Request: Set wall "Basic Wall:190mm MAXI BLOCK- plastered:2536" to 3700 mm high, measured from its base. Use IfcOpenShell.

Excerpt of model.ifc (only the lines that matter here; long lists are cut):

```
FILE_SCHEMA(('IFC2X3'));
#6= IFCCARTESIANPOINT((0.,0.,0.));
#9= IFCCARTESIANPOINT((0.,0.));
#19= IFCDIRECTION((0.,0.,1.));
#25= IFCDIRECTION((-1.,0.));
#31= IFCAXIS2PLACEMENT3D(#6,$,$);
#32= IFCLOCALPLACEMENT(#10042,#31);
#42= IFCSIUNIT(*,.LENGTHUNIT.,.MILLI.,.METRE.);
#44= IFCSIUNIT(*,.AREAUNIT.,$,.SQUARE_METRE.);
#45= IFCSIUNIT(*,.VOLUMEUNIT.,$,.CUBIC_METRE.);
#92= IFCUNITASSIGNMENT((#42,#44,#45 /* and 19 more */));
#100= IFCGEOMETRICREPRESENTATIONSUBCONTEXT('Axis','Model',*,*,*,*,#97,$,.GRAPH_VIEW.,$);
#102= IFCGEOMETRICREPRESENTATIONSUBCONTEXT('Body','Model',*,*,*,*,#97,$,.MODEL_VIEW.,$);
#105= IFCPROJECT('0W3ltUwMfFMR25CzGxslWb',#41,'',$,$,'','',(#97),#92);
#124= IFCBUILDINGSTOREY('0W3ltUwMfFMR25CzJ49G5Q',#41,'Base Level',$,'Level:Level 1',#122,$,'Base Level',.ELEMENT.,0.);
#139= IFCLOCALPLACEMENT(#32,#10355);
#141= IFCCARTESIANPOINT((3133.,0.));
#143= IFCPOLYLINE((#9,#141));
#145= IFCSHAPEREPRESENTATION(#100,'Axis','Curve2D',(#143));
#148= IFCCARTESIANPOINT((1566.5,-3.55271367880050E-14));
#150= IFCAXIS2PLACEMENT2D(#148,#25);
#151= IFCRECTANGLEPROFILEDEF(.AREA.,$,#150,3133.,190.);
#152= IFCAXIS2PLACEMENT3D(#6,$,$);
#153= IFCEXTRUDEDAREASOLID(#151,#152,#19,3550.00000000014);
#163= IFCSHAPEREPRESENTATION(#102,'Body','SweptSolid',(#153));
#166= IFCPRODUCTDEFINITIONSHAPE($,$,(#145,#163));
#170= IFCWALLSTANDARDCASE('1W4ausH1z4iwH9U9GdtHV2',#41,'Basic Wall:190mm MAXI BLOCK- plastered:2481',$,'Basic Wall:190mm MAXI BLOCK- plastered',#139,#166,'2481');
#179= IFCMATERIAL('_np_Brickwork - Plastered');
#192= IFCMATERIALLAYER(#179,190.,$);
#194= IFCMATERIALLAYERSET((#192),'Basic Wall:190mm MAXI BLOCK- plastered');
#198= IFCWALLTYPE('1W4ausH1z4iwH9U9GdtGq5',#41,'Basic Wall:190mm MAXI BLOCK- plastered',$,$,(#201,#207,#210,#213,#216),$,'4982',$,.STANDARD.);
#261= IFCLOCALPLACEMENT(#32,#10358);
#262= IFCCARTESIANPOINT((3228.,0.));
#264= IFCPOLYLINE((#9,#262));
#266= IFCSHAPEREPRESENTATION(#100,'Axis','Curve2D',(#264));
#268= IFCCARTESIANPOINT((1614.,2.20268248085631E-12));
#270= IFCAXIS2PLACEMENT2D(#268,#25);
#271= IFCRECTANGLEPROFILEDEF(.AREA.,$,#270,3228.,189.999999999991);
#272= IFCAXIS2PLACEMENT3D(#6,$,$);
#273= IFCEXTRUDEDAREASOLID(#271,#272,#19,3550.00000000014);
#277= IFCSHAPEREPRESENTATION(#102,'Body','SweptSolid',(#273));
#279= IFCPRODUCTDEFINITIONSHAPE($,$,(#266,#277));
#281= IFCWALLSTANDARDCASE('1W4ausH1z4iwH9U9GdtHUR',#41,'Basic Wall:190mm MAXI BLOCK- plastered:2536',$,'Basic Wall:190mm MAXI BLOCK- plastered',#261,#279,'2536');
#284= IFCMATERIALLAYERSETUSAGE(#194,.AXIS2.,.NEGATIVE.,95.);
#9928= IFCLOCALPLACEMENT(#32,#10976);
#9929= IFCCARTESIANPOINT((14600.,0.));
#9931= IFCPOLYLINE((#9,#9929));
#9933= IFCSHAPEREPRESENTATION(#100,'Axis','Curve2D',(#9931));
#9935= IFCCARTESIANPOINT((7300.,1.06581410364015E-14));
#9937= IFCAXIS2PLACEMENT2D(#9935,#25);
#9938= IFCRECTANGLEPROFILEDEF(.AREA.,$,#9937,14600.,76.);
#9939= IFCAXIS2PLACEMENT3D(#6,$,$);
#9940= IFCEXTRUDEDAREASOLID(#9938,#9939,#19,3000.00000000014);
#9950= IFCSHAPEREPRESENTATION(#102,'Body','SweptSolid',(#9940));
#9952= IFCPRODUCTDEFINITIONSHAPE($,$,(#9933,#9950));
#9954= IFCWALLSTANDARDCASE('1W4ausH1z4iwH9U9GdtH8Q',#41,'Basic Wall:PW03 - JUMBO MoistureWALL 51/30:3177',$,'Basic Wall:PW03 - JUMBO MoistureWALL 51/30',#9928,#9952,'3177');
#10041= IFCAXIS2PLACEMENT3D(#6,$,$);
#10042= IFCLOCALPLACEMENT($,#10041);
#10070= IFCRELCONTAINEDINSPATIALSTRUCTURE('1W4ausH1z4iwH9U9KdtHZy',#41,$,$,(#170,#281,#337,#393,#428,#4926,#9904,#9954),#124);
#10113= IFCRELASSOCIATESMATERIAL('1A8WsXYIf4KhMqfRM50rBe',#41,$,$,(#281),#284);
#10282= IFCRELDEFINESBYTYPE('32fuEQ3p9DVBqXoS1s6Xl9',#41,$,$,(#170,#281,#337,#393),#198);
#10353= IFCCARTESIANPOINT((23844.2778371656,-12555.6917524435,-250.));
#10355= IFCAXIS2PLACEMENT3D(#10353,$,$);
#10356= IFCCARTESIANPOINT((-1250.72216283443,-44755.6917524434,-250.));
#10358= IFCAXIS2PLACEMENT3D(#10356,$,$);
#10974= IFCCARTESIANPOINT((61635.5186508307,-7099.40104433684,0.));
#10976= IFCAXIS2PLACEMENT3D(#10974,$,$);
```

```python
import ifcopenshell
import ifcopenshell.geom
import ifcopenshell.util.representation
import ifcopenshell.util.shape
import ifcopenshell.util.unit

model = ifcopenshell.open("model.ifc")
unit_scale = ifcopenshell.util.unit.calculate_unit_scale(model)
settings = ifcopenshell.geom.settings()


def volume(element):
    """Net volume in cubic metres, openings subtracted."""
    shape = ifcopenshell.geom.create_shape(settings, element)
    return ifcopenshell.util.shape.get_volume(shape.geometry)


wall = model.by_guid("1W4ausH1z4iwH9U9GdtHUR")
before = volume(wall)

body = ifcopenshell.util.representation.get_representation(wall, "Model", "Body")
solid = body.Items[0]
old_height = solid.Depth
solid.Depth = 3.7 / unit_scale
after = volume(wall)

print(f"height {old_height:g} -> {solid.Depth:g}, volume {before:.3f} -> {after:.3f} m3")

model.write("model_updated.ifc")
```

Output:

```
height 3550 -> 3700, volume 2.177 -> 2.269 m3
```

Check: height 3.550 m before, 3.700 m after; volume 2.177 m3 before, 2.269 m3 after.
